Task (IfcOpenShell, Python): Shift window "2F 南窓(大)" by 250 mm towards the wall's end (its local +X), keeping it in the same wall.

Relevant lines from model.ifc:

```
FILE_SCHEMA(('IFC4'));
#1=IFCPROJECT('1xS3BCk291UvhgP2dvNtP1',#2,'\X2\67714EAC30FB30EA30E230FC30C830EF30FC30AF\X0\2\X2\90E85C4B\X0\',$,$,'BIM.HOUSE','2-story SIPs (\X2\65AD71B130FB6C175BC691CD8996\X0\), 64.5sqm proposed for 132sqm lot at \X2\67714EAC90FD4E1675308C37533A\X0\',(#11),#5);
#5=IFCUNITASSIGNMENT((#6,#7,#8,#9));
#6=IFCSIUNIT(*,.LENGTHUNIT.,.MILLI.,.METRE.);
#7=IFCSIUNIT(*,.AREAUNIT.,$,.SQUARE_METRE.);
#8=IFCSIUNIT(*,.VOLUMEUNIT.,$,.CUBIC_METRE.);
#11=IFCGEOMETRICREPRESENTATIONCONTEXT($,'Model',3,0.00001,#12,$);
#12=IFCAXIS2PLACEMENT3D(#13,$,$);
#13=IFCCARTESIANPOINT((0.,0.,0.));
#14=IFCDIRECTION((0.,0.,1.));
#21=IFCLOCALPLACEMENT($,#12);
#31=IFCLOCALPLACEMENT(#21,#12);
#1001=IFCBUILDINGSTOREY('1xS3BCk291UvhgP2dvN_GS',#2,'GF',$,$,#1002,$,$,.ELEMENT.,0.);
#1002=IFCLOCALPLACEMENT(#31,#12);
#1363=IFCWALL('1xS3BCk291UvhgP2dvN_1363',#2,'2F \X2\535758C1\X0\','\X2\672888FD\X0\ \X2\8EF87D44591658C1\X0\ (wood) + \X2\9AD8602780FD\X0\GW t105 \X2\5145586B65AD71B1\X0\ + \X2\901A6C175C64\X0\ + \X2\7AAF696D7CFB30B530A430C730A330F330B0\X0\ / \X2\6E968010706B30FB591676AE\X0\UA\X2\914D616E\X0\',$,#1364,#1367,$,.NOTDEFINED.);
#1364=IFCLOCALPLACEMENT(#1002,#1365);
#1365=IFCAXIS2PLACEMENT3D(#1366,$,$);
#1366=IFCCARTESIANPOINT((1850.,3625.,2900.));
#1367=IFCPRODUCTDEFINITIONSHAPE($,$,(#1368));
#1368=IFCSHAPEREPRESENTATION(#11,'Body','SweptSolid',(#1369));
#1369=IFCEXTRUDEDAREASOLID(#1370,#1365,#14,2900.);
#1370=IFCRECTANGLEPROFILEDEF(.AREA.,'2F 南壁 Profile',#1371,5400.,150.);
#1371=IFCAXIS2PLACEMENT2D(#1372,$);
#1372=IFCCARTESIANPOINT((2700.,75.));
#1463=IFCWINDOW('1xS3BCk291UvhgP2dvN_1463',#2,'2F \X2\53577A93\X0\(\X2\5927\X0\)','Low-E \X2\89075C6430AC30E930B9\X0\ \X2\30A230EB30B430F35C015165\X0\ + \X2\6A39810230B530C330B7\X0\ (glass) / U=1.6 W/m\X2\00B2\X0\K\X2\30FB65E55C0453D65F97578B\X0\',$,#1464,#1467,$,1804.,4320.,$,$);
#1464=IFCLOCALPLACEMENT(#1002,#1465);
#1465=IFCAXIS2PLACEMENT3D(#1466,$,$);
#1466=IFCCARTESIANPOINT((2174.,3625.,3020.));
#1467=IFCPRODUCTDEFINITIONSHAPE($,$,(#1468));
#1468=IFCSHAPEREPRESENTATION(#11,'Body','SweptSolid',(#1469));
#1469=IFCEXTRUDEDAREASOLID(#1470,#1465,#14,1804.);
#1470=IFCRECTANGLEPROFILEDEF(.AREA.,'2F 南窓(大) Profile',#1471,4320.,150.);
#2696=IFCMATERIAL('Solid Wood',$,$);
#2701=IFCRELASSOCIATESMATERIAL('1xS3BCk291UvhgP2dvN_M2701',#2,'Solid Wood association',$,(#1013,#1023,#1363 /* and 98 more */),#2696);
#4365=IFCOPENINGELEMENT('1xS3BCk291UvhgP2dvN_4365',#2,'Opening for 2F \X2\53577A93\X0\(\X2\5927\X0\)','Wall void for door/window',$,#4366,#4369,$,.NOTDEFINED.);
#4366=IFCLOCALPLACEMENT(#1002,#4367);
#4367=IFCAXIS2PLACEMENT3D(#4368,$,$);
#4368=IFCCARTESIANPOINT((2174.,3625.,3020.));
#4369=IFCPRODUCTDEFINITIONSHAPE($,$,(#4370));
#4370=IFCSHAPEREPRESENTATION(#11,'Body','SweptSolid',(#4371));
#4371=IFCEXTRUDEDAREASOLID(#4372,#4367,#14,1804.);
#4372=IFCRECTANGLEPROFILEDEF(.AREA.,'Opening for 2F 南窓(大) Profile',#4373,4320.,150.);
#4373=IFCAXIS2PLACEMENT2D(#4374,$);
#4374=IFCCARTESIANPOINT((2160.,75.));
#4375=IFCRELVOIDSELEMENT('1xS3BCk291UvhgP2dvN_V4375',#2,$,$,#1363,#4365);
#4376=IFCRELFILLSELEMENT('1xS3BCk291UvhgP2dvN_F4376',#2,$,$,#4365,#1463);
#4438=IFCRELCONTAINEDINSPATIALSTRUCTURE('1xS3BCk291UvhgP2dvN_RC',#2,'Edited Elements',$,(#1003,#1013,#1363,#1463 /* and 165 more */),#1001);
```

```python
import ifcopenshell
import ifcopenshell.api.geometry
import ifcopenshell.util.placement

model = ifcopenshell.open("model.ifc")

window = model.by_guid("1xS3BCk291UvhgP2dvN_1463")
opening = window.FillsVoids[0].RelatingOpeningElement
wall = opening.VoidsElements[0].RelatingBuildingElement

wall_matrix = ifcopenshell.util.placement.get_local_placement(wall.ObjectPlacement)
shift = wall_matrix[:3, 0] * 250.0
before = ifcopenshell.util.placement.get_local_placement(window.ObjectPlacement)[:3, 3].copy()

# The window is not placed relative to its opening, so move both.
for product in (opening, window):
    matrix = ifcopenshell.util.placement.get_local_placement(product.ObjectPlacement)
    matrix[:3, 3] += shift
    ifcopenshell.api.geometry.edit_object_placement(model, product=product, matrix=matrix, is_si=False)

after = ifcopenshell.util.placement.get_local_placement(window.ObjectPlacement)[:3, 3]
print("window moved by", (after - before).round(3) + 0.0)

model.write("model-out.ifc")
```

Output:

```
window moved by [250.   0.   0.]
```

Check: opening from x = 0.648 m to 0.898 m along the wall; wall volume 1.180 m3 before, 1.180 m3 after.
